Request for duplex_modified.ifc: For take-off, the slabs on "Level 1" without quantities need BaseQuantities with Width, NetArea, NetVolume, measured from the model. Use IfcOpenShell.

First a look at what the model holds.

```python
import ifcopenshell
import ifcopenshell.util.element
import ifcopenshell.util.unit

model = ifcopenshell.open("duplex_modified.ifc")
print(model.schema)
for unit_type in ("LENGTHUNIT", "AREAUNIT", "VOLUMEUNIT"):
    print(unit_type, ifcopenshell.util.unit.calculate_unit_scale(model, unit_type))
storey = next(s for s in model.by_type("IfcBuildingStorey") if s.Name == "Level 1")
slabs = [e for e in ifcopenshell.util.element.get_decomposition(storey) if e.is_a("IfcSlab")]
for e in sorted(slabs, key=lambda e: e.id()):
    print(e.id(), e.is_a(), e.Name, list(ifcopenshell.util.element.get_psets(e, qtos_only=True)), sep=" | ")
```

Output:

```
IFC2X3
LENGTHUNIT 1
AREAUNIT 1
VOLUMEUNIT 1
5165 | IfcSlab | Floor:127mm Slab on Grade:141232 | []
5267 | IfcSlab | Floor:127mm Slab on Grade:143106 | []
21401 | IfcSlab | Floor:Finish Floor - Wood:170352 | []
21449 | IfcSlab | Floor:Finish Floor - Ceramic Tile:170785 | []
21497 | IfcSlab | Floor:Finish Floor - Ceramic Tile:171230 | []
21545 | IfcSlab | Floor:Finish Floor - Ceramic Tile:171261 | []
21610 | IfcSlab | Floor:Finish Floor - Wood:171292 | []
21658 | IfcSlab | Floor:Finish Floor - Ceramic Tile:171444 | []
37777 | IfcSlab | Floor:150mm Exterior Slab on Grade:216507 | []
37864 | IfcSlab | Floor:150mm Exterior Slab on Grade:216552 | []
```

```python
import ifcopenshell
import ifcopenshell.api.pset
import ifcopenshell.geom
import ifcopenshell.util.element
import ifcopenshell.util.shape
import ifcopenshell.util.unit

model = ifcopenshell.open("duplex_modified.ifc")
unit_scale = ifcopenshell.util.unit.calculate_unit_scale(model)
area_scale = ifcopenshell.util.unit.calculate_unit_scale(model, "AREAUNIT")
volume_scale = ifcopenshell.util.unit.calculate_unit_scale(model, "VOLUMEUNIT")
settings = ifcopenshell.geom.settings()

storey = next(s for s in model.by_type("IfcBuildingStorey") if s.Name == "Level 1")
slabs = [e for e in ifcopenshell.util.element.get_decomposition(storey) if e.is_a("IfcSlab")]

for e in sorted(slabs, key=lambda e: e.id()):
    if ifcopenshell.util.element.get_psets(e, qtos_only=True, should_inherit=False):
        continue
    # Geometry comes back in metres, in the element's own axes.
    shape = ifcopenshell.geom.create_shape(settings, e)
    values = {
        "Width": ifcopenshell.util.shape.get_z(shape.geometry) / unit_scale,
        "NetArea": ifcopenshell.util.shape.get_footprint_area(shape.geometry) / area_scale,
        "NetVolume": ifcopenshell.util.shape.get_volume(shape.geometry) / volume_scale,
    }
    qto = ifcopenshell.api.pset.add_qto(model, product=e, name="BaseQuantities")
    ifcopenshell.api.pset.edit_qto(model, qto=qto, properties=values)
    print(e.id(), {k: round(v, 3) for k, v in values.items()})

model.write("duplex_modified_edited.ifc")
```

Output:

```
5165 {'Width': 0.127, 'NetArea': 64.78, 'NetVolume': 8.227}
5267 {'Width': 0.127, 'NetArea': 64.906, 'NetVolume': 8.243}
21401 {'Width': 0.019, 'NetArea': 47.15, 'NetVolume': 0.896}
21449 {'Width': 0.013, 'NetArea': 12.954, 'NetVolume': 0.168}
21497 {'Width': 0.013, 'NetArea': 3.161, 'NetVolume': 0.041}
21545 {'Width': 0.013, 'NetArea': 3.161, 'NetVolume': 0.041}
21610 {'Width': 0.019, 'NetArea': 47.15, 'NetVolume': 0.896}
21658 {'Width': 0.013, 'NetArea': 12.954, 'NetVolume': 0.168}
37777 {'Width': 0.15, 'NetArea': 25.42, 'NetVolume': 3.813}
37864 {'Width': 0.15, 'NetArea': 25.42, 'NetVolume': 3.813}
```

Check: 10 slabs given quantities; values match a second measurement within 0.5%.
